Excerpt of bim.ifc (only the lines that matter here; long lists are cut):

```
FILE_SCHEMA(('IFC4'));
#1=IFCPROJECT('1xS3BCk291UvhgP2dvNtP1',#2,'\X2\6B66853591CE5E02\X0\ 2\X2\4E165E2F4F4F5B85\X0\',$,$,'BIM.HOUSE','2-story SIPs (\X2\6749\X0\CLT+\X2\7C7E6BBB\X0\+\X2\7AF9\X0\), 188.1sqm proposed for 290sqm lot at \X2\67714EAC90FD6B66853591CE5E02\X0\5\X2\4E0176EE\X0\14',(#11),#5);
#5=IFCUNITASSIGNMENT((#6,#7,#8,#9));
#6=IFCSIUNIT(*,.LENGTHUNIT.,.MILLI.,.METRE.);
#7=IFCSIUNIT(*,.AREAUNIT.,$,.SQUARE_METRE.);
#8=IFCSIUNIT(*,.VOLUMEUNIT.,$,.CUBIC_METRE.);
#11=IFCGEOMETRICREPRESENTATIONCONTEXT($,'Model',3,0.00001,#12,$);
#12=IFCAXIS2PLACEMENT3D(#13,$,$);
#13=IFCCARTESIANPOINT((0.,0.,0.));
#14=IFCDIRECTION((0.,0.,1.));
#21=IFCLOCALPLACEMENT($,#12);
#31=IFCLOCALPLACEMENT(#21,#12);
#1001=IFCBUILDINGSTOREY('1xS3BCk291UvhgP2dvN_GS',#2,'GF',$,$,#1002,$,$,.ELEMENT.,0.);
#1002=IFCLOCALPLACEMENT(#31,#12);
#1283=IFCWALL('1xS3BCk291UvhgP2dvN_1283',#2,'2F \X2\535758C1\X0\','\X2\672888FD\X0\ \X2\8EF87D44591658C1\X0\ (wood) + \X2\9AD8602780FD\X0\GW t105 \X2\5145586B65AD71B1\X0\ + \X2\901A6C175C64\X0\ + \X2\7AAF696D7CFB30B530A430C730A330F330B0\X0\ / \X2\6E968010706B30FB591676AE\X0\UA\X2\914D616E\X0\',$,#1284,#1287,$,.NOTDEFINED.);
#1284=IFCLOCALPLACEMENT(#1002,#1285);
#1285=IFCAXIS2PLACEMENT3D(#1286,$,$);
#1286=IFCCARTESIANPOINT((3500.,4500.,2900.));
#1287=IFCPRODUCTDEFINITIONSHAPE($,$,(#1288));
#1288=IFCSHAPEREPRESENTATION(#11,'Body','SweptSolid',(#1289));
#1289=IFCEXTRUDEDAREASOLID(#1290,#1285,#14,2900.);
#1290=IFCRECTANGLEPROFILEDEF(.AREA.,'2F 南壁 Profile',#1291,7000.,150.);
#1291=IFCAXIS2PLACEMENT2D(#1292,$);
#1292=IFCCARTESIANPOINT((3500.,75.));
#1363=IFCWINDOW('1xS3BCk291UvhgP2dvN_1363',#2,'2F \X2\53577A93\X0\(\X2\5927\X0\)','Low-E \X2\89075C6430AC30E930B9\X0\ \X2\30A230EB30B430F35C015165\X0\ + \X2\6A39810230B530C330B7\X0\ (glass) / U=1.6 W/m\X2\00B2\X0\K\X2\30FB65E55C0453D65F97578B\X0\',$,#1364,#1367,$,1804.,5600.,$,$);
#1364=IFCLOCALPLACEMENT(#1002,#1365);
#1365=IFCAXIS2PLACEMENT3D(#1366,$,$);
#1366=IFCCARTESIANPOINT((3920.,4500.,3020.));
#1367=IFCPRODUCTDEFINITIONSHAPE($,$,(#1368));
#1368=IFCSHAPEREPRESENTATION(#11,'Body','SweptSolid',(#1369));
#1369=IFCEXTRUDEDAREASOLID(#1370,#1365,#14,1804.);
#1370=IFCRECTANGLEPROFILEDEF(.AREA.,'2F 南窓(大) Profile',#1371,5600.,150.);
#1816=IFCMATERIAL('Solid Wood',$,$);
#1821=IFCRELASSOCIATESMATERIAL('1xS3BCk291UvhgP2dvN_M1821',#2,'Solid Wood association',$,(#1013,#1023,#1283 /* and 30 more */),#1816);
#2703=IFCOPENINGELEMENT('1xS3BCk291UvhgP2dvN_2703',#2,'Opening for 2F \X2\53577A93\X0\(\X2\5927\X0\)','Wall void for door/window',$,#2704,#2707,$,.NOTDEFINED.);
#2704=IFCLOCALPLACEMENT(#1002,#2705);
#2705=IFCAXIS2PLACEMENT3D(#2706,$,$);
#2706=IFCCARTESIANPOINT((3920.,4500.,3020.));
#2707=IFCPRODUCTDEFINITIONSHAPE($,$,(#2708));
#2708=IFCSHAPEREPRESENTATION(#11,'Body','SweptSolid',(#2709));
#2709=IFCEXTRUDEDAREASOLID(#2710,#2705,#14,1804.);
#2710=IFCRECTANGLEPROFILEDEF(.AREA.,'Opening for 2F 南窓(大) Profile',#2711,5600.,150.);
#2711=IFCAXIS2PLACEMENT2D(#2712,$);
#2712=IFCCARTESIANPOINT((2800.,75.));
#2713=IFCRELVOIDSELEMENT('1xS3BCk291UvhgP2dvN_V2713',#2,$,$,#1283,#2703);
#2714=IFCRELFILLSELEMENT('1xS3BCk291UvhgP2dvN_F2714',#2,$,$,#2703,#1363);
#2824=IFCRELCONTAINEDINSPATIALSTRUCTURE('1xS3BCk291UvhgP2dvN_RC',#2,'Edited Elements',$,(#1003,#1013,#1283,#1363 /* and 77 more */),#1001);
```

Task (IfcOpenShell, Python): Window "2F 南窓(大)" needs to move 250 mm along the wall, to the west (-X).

```python
import ifcopenshell
import ifcopenshell.api.geometry
import ifcopenshell.util.placement
import ifcopenshell.util.unit

model = ifcopenshell.open("bim.ifc")
unit_scale = ifcopenshell.util.unit.calculate_unit_scale(model)

window = model.by_guid("1xS3BCk291UvhgP2dvN_1363")
opening = window.FillsVoids[0].RelatingOpeningElement
wall = opening.VoidsElements[0].RelatingBuildingElement

wall_matrix = ifcopenshell.util.placement.get_local_placement(wall.ObjectPlacement)
shift = wall_matrix[:3, 0] * -0.25 / unit_scale
before = ifcopenshell.util.placement.get_local_placement(window.ObjectPlacement)[:3, 3].copy()

# The window is not placed relative to its opening, so move both.
for product in (opening, window):
    matrix = ifcopenshell.util.placement.get_local_placement(product.ObjectPlacement)
    matrix[:3, 3] += shift
    ifcopenshell.api.geometry.edit_object_placement(model, product=product, matrix=matrix, is_si=False)

after = ifcopenshell.util.placement.get_local_placement(window.ObjectPlacement)[:3, 3]
print("window moved by", (after - before).round(3) + 0.0)

model.write("bim_rev.ifc")
```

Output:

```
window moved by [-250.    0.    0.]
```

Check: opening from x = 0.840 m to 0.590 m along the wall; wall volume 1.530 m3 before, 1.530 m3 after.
